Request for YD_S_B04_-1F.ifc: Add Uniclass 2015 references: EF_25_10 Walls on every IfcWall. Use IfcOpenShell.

First a look at what the model holds.

```python
import ifcopenshell

model = ifcopenshell.open("YD_S_B04_-1F.ifc")
print(model.schema)
print("classifications:", [c.Name for c in model.by_type("IfcClassification")])
for ifc_class in ("IfcDoor", "IfcRoof", "IfcStair", "IfcWall", "IfcWindow"):
    print(ifc_class, len(model.by_type(ifc_class)))
```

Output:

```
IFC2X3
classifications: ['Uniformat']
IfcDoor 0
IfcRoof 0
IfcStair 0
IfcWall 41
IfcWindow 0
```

```python
import ifcopenshell
import ifcopenshell.api.classification

model = ifcopenshell.open("YD_S_B04_-1F.ifc")

# IFC2X3 requires Source and Edition and has no link from the project to the system.
system = model.create_entity("IfcClassification", Source="NBS", Edition="2015", Name="Uniclass 2015")

codes = {
    "IfcWall": ("EF_25_10", "Walls"),
}
for ifc_class, (code, name) in codes.items():
    products = model.by_type(ifc_class)
    ifcopenshell.api.classification.add_reference(
        model, products=products, classification=system, identification=code, name=name
    )
    print(code, len(products))

model.write("YD_S_B04_-1F_updated.ifc")
```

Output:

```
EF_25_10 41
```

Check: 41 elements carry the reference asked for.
